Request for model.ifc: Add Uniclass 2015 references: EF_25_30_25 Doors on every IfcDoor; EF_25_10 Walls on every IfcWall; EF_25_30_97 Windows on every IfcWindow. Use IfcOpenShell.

First a look at what the model holds.

```python
import ifcopenshell

model = ifcopenshell.open("model.ifc")
print(model.schema)
print("classifications:", [c.Name for c in model.by_type("IfcClassification")])
for ifc_class in ("IfcDoor", "IfcRoof", "IfcStair", "IfcWall", "IfcWindow"):
    print(ifc_class, len(model.by_type(ifc_class)))
```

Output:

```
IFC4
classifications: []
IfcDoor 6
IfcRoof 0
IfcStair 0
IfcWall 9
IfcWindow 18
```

```python
import ifcopenshell
import ifcopenshell.api.classification

model = ifcopenshell.open("model.ifc")

system = ifcopenshell.api.classification.add_classification(model, classification="Uniclass 2015")

codes = {
    "IfcDoor": ("EF_25_30_25", "Doors"),
    "IfcWall": ("EF_25_10", "Walls"),
    "IfcWindow": ("EF_25_30_97", "Windows"),
}
for ifc_class, (code, name) in codes.items():
    products = model.by_type(ifc_class)
    ifcopenshell.api.classification.add_reference(
        model, products=products, classification=system, identification=code, name=name
    )
    print(code, len(products))

model.write("model_updated.ifc")
```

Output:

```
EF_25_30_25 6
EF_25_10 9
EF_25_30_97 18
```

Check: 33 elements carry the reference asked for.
